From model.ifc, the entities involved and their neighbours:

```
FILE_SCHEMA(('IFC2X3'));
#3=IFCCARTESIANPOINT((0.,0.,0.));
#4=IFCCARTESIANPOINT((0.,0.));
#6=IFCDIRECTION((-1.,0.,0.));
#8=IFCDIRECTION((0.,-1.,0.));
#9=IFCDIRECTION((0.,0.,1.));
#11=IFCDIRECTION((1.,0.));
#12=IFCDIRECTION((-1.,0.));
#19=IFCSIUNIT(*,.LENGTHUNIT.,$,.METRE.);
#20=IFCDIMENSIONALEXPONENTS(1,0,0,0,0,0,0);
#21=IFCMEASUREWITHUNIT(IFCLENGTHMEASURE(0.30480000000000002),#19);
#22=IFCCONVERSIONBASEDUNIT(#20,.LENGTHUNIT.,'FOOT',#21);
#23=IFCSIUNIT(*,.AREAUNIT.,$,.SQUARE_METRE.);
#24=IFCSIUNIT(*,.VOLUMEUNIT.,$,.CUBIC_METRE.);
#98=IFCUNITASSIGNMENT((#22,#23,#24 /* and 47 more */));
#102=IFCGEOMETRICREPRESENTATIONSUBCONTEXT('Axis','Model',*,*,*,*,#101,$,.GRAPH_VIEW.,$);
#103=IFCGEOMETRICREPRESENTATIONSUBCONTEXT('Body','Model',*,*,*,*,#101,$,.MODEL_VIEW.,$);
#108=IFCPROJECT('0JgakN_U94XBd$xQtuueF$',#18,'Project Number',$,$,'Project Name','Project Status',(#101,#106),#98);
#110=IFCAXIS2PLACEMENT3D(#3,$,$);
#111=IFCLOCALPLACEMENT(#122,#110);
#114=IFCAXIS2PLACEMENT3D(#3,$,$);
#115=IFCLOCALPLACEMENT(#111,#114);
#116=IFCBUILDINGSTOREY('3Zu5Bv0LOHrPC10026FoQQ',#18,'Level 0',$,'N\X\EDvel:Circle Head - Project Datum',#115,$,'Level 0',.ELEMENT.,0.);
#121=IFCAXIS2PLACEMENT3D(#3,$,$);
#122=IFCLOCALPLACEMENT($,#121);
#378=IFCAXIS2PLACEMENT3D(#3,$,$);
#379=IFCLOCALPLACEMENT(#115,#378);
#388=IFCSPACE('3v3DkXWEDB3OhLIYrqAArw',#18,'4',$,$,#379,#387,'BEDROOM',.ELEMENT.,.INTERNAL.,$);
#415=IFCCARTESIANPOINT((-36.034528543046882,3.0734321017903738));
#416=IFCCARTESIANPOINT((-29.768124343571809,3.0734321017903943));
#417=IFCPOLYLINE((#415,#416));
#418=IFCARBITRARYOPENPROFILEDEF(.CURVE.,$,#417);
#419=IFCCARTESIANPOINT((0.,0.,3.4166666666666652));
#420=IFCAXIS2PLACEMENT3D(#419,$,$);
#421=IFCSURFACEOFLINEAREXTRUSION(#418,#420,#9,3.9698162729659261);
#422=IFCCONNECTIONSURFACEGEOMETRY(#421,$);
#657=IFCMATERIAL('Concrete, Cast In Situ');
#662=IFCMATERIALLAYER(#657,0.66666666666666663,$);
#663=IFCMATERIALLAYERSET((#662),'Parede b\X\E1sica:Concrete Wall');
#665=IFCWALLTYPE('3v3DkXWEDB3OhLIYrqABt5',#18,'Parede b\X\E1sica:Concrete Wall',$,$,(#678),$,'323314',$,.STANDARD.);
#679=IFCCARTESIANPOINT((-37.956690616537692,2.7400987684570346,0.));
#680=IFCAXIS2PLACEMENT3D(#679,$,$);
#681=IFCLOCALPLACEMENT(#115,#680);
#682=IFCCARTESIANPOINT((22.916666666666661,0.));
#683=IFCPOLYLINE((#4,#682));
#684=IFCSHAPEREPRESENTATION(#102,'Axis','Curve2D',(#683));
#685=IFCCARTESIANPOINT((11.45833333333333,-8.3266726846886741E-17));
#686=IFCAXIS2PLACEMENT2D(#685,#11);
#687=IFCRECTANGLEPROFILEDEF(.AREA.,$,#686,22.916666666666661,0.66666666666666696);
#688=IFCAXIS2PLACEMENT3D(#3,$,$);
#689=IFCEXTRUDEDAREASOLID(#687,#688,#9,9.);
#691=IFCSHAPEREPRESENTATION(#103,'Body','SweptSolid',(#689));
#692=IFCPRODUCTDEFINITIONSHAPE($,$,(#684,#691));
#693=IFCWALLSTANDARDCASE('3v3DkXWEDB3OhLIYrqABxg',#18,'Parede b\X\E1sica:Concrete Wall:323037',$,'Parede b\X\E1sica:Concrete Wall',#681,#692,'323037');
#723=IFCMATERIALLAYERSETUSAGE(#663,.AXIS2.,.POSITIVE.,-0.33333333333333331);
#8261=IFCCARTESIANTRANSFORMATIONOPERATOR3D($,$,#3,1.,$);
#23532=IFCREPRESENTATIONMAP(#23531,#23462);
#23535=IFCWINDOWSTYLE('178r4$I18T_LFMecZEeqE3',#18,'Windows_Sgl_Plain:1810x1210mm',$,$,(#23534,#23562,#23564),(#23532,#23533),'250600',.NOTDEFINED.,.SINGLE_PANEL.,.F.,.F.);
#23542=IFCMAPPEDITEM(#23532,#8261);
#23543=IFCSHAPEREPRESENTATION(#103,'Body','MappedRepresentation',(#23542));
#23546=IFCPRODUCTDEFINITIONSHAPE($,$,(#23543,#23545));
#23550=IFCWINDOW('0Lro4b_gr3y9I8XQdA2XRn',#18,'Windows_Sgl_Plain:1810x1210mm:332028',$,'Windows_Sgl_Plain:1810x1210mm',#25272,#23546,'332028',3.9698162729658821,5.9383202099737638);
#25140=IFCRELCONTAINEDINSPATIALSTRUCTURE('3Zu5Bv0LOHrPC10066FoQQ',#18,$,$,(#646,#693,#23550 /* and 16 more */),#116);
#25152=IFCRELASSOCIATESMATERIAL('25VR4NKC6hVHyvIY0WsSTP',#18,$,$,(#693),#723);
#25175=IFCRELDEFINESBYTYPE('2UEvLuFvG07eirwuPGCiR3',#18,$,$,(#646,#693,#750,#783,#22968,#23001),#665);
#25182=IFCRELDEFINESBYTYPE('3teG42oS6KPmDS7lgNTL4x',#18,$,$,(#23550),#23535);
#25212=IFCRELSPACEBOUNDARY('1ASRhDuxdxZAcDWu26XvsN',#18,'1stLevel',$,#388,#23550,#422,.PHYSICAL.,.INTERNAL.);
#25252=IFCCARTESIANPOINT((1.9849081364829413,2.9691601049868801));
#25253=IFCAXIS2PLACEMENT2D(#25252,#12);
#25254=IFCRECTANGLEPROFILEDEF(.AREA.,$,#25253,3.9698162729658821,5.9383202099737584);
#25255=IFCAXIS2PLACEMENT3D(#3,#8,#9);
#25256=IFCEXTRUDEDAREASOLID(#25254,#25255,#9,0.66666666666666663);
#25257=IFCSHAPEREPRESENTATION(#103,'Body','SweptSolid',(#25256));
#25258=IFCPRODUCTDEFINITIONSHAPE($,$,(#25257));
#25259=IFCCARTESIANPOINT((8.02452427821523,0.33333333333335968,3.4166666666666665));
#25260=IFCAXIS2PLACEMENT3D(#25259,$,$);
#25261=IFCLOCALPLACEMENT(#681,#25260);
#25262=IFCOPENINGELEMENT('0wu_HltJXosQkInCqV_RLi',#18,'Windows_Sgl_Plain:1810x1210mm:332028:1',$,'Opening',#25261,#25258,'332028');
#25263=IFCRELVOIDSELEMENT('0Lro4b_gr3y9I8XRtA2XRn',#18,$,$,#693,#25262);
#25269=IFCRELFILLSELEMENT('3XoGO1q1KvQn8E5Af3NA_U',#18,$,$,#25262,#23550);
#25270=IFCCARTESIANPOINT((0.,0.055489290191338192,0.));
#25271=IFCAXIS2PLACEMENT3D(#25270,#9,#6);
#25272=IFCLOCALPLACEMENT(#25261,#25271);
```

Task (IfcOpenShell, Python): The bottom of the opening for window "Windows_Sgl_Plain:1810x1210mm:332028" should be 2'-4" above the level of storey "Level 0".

```python
import numpy as np
import ifcopenshell
import ifcopenshell.api.geometry
import ifcopenshell.geom
import ifcopenshell.util.element
import ifcopenshell.util.placement
import ifcopenshell.util.shape
import ifcopenshell.util.unit

model = ifcopenshell.open("model.ifc")
unit_scale = ifcopenshell.util.unit.calculate_unit_scale(model)

window = model.by_id(23550)
opening = window.FillsVoids[0].RelatingOpeningElement
storey = ifcopenshell.util.element.get_container(window, ifc_class="IfcBuildingStorey")
level = ifcopenshell.util.placement.get_local_placement(storey.ObjectPlacement)[2, 3]

# The opening's origin need not be at the sill, so measure its lowest point.
shape = ifcopenshell.geom.create_shape(ifcopenshell.geom.settings(), opening)
bottom = ifcopenshell.util.shape.get_shape_bottom_elevation(shape, shape.geometry) / unit_scale
dz = level + 28 * 0.0254 / unit_scale - bottom

shift = np.array([0.0, 0.0, dz])
# The window is placed relative to its opening, so it follows when the opening moves.
matrix = ifcopenshell.util.placement.get_local_placement(opening.ObjectPlacement)
matrix[:3, 3] += shift
ifcopenshell.api.geometry.edit_object_placement(
    model, product=opening, matrix=matrix, is_si=False, should_transform_children=True
)

# Space boundary surfaces are stored in each space's coordinates; move them too.
for rel in window.ProvidesBoundaries:
    if not rel.ConnectionGeometry:
        continue
    surface = rel.ConnectionGeometry.SurfaceOnRelatingElement
    space_matrix = ifcopenshell.util.placement.get_local_placement(rel.RelatingSpace.ObjectPlacement)
    point = np.array(surface.Position.Location.Coordinates) + space_matrix[:3, :3].T @ shift
    surface.Position = model.createIfcAxis2Placement3D(
        model.createIfcCartesianPoint(point.tolist()), surface.Position.Axis, surface.Position.RefDirection
    )

print(f"moved by {dz * unit_scale:+.3f} m")

model.write("model_v2.ifc")
```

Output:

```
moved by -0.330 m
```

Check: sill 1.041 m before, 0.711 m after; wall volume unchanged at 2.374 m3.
